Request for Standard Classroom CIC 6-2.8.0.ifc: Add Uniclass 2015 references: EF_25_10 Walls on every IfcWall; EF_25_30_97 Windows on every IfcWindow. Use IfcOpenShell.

First a look at what the model holds.

```python
import ifcopenshell

model = ifcopenshell.open("Standard Classroom CIC 6-2.8.0.ifc")
print(model.schema)
print("classifications:", [c.Name for c in model.by_type("IfcClassification")])
for ifc_class in ("IfcDoor", "IfcRoof", "IfcStair", "IfcWall", "IfcWindow"):
    print(ifc_class, len(model.by_type(ifc_class)))
```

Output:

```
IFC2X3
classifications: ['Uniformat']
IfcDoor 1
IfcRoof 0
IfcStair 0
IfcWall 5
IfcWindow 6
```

```python
import ifcopenshell
import ifcopenshell.api.classification

model = ifcopenshell.open("Standard Classroom CIC 6-2.8.0.ifc")

# IFC2X3 requires Source and Edition and has no link from the project to the system.
system = model.create_entity("IfcClassification", Source="NBS", Edition="2015", Name="Uniclass 2015")

codes = {
    "IfcWall": ("EF_25_10", "Walls"),
    "IfcWindow": ("EF_25_30_97", "Windows"),
}
for ifc_class, (code, name) in codes.items():
    products = model.by_type(ifc_class)
    ifcopenshell.api.classification.add_reference(
        model, products=products, classification=system, identification=code, name=name
    )
    print(code, len(products))

model.write("Standard Classroom CIC 6-2.8.0_updated.ifc")
```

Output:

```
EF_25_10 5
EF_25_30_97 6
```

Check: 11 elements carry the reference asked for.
